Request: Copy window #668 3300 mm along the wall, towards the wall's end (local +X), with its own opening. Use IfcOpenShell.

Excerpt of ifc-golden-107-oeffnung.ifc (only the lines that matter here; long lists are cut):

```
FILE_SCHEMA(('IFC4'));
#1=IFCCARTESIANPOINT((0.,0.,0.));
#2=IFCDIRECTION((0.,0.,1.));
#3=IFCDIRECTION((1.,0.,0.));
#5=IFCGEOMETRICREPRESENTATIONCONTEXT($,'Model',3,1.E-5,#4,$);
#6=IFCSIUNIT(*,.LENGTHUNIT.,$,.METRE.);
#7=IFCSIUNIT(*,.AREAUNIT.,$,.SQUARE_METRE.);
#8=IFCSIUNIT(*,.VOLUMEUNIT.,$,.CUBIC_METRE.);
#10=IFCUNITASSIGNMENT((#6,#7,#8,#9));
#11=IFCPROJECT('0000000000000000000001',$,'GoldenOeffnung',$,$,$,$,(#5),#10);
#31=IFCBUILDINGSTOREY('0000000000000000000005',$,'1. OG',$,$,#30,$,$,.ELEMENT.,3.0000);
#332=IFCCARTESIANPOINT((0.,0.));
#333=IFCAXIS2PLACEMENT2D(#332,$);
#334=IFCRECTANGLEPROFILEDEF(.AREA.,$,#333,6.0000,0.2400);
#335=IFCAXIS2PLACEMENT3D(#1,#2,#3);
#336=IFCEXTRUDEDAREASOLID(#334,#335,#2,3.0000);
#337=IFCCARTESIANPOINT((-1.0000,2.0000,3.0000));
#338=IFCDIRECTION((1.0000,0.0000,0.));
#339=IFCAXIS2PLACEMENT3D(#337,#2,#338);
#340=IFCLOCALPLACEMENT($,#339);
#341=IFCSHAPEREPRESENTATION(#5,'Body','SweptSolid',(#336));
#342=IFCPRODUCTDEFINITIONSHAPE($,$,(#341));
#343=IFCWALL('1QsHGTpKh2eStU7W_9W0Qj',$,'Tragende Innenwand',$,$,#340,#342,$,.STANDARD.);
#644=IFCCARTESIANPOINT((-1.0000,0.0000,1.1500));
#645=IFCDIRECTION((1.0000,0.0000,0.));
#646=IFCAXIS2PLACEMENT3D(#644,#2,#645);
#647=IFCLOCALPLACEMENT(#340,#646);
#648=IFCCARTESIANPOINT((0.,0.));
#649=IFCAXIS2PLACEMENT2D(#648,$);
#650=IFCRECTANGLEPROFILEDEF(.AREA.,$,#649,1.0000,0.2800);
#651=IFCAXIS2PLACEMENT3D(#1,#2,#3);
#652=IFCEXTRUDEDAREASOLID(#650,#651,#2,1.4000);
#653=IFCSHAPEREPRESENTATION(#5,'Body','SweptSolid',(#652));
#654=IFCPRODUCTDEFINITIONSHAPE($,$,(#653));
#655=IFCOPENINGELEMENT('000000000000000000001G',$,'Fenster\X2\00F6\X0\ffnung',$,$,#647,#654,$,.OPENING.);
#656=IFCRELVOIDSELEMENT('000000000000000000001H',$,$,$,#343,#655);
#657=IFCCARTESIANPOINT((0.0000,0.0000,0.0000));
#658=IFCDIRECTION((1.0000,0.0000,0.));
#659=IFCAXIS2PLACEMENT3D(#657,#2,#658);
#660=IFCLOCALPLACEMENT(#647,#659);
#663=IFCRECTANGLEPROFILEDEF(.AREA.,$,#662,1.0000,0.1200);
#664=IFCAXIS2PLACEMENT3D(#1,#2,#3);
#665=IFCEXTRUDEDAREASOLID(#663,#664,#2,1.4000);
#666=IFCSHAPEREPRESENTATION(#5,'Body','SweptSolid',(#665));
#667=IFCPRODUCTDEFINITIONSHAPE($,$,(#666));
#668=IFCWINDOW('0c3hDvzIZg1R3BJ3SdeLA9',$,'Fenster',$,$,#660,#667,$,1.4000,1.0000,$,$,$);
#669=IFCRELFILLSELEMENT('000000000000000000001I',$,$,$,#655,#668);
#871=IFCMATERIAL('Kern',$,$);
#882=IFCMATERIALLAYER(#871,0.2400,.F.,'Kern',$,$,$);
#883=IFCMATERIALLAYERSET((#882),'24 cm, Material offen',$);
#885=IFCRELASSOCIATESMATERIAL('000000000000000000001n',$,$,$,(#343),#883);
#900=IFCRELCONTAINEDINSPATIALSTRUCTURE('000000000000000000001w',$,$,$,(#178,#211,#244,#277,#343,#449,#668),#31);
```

```python
import ifcopenshell
import ifcopenshell.api.feature
import ifcopenshell.api.geometry
import ifcopenshell.api.root
import ifcopenshell.geom
import ifcopenshell.util.element
import ifcopenshell.util.placement
import ifcopenshell.util.shape

model = ifcopenshell.open("ifc-golden-107-oeffnung.ifc")
settings = ifcopenshell.geom.settings()


def volume(element):
    """Net volume in cubic metres, openings subtracted."""
    shape = ifcopenshell.geom.create_shape(settings, element)
    return ifcopenshell.util.shape.get_volume(shape.geometry)


window = model.by_guid("0c3hDvzIZg1R3BJ3SdeLA9")
opening = window.FillsVoids[0].RelatingOpeningElement
wall = opening.VoidsElements[0].RelatingBuildingElement
before = volume(wall)
shift = ifcopenshell.util.placement.get_local_placement(wall.ObjectPlacement)[:3, 0] * 3.3

# copy_class copies the void relationship, type, container and properties, but no geometry.
new_opening = ifcopenshell.api.root.copy_class(model, product=opening)
new_opening.Representation = ifcopenshell.util.element.copy_deep(
    model, opening.Representation, exclude=["IfcGeometricRepresentationContext", "IfcRepresentationMap"]
)
new_window = ifcopenshell.api.root.copy_class(model, product=window)
new_window.Representation = ifcopenshell.util.element.copy_deep(
    model, window.Representation, exclude=["IfcGeometricRepresentationContext", "IfcRepresentationMap"]
)
ifcopenshell.api.feature.add_filling(model, opening=new_opening, element=new_window)

for old, new in ((opening, new_opening), (window, new_window)):
    matrix = ifcopenshell.util.placement.get_local_placement(old.ObjectPlacement)
    matrix[:3, 3] += shift
    ifcopenshell.api.geometry.edit_object_placement(model, product=new, matrix=matrix, is_si=False)

after = volume(wall)

print(f"wall volume {before:.3f} -> {after:.3f} m3")

model.write("ifc-golden-107-oeffnung_v2.ifc")
```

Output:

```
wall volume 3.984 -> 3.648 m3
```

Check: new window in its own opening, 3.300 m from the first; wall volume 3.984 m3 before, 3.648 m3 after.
